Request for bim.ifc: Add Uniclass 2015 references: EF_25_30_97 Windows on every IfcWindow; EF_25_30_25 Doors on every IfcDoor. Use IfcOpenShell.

First a look at what the model holds.

```python
import ifcopenshell

model = ifcopenshell.open("bim.ifc")
print(model.schema)
print("classifications:", [c.Name for c in model.by_type("IfcClassification")])
for ifc_class in ("IfcDoor", "IfcRoof", "IfcStair", "IfcWall", "IfcWindow"):
    print(ifc_class, len(model.by_type(ifc_class)))
```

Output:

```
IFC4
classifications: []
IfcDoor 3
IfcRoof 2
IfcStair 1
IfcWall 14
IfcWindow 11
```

```python
import ifcopenshell
import ifcopenshell.api.classification

model = ifcopenshell.open("bim.ifc")

system = ifcopenshell.api.classification.add_classification(model, classification="Uniclass 2015")

codes = {
    "IfcWindow": ("EF_25_30_97", "Windows"),
    "IfcDoor": ("EF_25_30_25", "Doors"),
}
for ifc_class, (code, name) in codes.items():
    products = model.by_type(ifc_class)
    ifcopenshell.api.classification.add_reference(
        model, products=products, classification=system, identification=code, name=name
    )
    print(code, len(products))

model.write("bim_edited.ifc")
```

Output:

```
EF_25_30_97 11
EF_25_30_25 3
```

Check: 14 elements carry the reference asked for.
